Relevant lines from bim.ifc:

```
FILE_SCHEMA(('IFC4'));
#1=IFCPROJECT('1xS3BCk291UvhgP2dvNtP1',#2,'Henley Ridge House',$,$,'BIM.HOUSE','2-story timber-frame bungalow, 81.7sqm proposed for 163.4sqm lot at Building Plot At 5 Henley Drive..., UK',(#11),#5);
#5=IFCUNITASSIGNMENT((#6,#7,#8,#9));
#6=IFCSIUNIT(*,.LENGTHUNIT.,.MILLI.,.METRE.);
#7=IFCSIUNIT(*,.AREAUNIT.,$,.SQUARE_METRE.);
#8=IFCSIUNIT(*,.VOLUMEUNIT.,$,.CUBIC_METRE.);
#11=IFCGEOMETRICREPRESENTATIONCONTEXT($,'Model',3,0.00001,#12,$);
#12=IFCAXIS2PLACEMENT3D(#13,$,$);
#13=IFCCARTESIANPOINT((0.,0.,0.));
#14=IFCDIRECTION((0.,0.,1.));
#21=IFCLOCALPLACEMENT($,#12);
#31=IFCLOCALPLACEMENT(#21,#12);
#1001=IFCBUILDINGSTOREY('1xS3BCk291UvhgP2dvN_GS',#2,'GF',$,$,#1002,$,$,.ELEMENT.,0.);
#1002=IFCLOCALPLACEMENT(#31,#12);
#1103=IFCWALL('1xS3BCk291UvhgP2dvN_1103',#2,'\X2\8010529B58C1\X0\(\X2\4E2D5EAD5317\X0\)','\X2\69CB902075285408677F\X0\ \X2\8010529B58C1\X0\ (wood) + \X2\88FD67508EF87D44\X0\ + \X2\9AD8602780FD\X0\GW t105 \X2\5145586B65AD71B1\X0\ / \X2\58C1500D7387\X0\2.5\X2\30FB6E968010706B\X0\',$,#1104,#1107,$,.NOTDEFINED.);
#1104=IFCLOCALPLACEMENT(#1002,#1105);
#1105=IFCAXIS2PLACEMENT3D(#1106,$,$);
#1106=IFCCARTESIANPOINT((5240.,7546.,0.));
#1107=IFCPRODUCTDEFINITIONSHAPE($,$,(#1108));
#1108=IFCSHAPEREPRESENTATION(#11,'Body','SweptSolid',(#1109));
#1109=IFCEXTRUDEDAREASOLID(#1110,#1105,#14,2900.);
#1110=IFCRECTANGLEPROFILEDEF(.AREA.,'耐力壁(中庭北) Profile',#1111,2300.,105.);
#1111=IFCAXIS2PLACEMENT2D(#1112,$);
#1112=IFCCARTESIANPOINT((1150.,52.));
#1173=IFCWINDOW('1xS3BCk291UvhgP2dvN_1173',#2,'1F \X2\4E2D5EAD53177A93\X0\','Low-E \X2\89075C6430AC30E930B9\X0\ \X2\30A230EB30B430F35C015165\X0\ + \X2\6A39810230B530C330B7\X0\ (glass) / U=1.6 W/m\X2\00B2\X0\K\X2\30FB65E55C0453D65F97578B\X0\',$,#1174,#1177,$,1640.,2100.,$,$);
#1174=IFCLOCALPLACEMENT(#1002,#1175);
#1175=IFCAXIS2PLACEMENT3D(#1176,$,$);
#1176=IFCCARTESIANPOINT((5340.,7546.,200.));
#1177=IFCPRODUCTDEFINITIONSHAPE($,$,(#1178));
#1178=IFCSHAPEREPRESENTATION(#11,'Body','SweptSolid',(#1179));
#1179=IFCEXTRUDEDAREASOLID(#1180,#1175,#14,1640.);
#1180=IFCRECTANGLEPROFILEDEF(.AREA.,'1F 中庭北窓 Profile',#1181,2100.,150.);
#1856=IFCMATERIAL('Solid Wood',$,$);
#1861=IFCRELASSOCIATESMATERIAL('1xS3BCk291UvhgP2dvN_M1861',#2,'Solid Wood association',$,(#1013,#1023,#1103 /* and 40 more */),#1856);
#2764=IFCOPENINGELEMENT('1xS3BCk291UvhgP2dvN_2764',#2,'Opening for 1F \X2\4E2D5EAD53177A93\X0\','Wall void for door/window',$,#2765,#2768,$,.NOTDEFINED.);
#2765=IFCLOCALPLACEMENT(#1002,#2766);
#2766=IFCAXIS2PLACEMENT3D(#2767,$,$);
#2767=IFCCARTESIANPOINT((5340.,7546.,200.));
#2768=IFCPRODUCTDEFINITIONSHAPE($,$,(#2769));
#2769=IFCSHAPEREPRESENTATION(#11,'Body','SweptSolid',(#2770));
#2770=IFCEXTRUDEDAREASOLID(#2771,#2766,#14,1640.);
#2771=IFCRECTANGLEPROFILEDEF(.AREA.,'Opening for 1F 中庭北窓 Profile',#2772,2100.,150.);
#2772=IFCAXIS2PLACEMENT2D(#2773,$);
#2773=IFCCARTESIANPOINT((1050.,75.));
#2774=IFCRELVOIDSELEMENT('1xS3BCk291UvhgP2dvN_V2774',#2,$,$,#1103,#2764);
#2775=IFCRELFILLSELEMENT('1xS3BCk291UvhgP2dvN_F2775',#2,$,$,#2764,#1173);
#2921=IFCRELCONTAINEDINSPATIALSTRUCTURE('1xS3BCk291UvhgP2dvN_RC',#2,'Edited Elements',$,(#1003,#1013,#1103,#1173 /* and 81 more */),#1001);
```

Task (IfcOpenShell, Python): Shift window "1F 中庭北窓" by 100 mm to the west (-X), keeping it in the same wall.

```python
import ifcopenshell
import ifcopenshell.api.geometry
import ifcopenshell.util.placement
import ifcopenshell.util.unit

model = ifcopenshell.open("bim.ifc")
unit_scale = ifcopenshell.util.unit.calculate_unit_scale(model)

window = model.by_guid("1xS3BCk291UvhgP2dvN_1173")
opening = window.FillsVoids[0].RelatingOpeningElement
wall = opening.VoidsElements[0].RelatingBuildingElement

wall_matrix = ifcopenshell.util.placement.get_local_placement(wall.ObjectPlacement)
shift = wall_matrix[:3, 0] * -0.1 / unit_scale
before = ifcopenshell.util.placement.get_local_placement(window.ObjectPlacement)[:3, 3].copy()

# The window is not placed relative to its opening, so move both.
for product in (opening, window):
    matrix = ifcopenshell.util.placement.get_local_placement(product.ObjectPlacement)
    matrix[:3, 3] += shift
    ifcopenshell.api.geometry.edit_object_placement(model, product=product, matrix=matrix, is_si=False)

after = ifcopenshell.util.placement.get_local_placement(window.ObjectPlacement)[:3, 3]
print("window moved by", (after - before).round(3) + 0.0)

model.write("bim-out.ifc")
```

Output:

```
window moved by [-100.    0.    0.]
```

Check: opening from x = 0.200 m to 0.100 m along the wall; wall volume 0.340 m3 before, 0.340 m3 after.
